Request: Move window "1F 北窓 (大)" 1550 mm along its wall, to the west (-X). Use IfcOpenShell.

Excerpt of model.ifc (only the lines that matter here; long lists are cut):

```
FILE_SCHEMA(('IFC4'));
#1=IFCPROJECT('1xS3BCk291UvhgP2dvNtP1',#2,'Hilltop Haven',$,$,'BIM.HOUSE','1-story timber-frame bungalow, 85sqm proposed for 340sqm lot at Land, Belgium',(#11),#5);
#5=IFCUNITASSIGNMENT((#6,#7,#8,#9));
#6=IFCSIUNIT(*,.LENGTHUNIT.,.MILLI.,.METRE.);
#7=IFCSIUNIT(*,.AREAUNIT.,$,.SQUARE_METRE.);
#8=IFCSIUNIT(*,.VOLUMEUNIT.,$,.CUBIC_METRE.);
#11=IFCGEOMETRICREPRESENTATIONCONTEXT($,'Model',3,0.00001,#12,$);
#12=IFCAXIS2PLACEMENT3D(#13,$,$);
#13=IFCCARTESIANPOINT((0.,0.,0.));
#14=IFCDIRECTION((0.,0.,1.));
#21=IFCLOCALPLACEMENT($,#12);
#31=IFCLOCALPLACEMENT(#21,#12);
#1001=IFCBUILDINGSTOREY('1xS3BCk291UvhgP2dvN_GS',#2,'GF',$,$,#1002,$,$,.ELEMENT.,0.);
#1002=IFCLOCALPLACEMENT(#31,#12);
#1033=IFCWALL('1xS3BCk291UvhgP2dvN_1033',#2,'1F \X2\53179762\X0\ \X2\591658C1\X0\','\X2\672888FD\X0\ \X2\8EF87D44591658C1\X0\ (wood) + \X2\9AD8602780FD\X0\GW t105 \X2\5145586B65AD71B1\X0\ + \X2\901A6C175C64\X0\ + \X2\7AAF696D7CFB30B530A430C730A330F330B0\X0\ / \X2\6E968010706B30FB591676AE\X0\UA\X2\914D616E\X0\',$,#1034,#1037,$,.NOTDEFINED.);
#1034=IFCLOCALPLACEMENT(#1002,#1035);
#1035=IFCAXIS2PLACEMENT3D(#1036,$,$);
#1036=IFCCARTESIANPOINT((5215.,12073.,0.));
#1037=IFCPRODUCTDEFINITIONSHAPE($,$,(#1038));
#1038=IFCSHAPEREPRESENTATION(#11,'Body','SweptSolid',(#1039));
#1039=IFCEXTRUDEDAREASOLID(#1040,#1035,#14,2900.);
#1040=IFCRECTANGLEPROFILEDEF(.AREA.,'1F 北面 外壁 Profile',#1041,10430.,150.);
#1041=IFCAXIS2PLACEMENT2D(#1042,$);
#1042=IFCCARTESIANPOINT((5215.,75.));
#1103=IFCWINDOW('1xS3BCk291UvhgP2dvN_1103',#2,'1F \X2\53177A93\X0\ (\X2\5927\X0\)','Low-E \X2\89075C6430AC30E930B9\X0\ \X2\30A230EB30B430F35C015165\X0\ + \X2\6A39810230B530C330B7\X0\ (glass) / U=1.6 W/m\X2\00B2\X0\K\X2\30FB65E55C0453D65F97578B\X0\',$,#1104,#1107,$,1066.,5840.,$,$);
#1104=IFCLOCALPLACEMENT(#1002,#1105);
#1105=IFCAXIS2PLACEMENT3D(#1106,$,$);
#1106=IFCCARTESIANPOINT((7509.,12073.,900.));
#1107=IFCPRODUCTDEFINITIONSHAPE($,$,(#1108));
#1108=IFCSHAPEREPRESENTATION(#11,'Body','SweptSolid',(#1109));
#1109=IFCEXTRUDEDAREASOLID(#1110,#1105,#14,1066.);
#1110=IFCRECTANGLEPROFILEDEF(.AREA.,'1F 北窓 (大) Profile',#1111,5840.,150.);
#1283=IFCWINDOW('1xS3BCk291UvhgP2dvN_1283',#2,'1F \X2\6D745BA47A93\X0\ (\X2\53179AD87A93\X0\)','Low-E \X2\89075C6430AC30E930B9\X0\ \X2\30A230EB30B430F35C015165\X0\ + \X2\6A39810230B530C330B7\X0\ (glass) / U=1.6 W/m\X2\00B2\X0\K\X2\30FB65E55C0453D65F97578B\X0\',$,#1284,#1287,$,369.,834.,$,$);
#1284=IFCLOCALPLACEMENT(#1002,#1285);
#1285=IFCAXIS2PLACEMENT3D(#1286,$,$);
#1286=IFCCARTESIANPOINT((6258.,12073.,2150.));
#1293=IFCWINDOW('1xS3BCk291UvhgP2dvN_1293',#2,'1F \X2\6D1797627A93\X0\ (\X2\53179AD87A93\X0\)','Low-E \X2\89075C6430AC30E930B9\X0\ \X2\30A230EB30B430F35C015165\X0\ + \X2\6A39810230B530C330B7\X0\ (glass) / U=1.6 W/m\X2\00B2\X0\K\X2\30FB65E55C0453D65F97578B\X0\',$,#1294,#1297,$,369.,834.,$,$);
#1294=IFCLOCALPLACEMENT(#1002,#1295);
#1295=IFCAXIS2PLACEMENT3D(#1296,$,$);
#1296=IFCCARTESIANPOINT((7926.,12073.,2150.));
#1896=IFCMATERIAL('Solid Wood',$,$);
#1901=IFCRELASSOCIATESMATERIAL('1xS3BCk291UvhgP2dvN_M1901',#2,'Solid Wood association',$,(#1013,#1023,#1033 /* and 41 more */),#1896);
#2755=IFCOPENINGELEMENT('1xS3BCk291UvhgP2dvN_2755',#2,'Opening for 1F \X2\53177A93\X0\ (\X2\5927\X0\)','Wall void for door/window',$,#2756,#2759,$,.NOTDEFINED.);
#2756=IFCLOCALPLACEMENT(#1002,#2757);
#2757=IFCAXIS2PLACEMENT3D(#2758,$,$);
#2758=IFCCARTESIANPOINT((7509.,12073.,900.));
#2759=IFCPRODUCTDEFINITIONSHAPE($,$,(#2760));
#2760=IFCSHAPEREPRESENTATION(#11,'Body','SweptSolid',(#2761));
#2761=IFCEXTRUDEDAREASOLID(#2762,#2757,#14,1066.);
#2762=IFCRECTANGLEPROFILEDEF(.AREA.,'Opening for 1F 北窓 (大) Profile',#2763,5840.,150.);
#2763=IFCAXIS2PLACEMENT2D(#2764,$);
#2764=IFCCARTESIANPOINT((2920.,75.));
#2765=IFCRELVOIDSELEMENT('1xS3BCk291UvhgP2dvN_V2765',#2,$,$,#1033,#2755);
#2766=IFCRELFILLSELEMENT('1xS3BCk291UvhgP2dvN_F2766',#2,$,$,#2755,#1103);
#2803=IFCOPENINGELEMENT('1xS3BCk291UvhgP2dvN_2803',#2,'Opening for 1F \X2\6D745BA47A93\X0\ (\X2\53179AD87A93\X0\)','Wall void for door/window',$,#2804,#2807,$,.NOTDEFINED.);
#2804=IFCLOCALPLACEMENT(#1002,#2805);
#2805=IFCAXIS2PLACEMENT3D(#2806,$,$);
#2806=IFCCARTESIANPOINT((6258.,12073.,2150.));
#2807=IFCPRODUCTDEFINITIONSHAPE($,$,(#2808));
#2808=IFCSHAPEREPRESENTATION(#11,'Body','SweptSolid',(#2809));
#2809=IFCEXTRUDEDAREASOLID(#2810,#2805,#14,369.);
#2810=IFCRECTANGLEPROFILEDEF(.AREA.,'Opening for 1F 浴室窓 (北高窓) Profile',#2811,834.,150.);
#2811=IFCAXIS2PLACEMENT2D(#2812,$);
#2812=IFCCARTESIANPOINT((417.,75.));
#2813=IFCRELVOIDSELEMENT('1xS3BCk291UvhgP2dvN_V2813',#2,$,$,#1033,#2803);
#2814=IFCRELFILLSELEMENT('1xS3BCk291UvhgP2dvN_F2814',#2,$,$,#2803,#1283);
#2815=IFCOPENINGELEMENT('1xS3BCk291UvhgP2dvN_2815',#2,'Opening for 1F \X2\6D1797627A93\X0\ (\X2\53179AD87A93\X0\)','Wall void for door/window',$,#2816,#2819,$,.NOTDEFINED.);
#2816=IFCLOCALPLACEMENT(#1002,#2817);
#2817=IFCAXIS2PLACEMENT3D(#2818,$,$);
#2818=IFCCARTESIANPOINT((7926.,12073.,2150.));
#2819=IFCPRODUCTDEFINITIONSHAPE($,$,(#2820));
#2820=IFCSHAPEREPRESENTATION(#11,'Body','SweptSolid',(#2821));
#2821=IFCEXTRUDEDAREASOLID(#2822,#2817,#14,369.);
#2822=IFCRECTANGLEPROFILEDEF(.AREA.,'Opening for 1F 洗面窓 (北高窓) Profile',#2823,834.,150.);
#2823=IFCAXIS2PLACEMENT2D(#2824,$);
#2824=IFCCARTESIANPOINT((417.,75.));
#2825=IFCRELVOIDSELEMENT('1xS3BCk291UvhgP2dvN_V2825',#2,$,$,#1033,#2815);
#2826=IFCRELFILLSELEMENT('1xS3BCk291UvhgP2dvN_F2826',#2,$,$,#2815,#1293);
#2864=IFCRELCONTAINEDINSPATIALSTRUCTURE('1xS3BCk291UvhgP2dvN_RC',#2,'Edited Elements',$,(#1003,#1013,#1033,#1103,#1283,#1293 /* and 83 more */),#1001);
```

```python
import ifcopenshell
import ifcopenshell.api.geometry
import ifcopenshell.util.placement

model = ifcopenshell.open("model.ifc")

window = model.by_guid("1xS3BCk291UvhgP2dvN_1103")
opening = window.FillsVoids[0].RelatingOpeningElement
wall = opening.VoidsElements[0].RelatingBuildingElement

wall_matrix = ifcopenshell.util.placement.get_local_placement(wall.ObjectPlacement)
shift = wall_matrix[:3, 0] * -1550.0
before = ifcopenshell.util.placement.get_local_placement(window.ObjectPlacement)[:3, 3].copy()

# The window is not placed relative to its opening, so move both.
for product in (opening, window):
    matrix = ifcopenshell.util.placement.get_local_placement(product.ObjectPlacement)
    matrix[:3, 3] += shift
    ifcopenshell.api.geometry.edit_object_placement(model, product=product, matrix=matrix, is_si=False)

after = ifcopenshell.util.placement.get_local_placement(window.ObjectPlacement)[:3, 3]
print("window moved by", (after - before).round(3) + 0.0)

model.write("model_rev.ifc")
```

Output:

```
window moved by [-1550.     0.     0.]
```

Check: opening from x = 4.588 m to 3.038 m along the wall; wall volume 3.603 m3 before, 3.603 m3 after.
